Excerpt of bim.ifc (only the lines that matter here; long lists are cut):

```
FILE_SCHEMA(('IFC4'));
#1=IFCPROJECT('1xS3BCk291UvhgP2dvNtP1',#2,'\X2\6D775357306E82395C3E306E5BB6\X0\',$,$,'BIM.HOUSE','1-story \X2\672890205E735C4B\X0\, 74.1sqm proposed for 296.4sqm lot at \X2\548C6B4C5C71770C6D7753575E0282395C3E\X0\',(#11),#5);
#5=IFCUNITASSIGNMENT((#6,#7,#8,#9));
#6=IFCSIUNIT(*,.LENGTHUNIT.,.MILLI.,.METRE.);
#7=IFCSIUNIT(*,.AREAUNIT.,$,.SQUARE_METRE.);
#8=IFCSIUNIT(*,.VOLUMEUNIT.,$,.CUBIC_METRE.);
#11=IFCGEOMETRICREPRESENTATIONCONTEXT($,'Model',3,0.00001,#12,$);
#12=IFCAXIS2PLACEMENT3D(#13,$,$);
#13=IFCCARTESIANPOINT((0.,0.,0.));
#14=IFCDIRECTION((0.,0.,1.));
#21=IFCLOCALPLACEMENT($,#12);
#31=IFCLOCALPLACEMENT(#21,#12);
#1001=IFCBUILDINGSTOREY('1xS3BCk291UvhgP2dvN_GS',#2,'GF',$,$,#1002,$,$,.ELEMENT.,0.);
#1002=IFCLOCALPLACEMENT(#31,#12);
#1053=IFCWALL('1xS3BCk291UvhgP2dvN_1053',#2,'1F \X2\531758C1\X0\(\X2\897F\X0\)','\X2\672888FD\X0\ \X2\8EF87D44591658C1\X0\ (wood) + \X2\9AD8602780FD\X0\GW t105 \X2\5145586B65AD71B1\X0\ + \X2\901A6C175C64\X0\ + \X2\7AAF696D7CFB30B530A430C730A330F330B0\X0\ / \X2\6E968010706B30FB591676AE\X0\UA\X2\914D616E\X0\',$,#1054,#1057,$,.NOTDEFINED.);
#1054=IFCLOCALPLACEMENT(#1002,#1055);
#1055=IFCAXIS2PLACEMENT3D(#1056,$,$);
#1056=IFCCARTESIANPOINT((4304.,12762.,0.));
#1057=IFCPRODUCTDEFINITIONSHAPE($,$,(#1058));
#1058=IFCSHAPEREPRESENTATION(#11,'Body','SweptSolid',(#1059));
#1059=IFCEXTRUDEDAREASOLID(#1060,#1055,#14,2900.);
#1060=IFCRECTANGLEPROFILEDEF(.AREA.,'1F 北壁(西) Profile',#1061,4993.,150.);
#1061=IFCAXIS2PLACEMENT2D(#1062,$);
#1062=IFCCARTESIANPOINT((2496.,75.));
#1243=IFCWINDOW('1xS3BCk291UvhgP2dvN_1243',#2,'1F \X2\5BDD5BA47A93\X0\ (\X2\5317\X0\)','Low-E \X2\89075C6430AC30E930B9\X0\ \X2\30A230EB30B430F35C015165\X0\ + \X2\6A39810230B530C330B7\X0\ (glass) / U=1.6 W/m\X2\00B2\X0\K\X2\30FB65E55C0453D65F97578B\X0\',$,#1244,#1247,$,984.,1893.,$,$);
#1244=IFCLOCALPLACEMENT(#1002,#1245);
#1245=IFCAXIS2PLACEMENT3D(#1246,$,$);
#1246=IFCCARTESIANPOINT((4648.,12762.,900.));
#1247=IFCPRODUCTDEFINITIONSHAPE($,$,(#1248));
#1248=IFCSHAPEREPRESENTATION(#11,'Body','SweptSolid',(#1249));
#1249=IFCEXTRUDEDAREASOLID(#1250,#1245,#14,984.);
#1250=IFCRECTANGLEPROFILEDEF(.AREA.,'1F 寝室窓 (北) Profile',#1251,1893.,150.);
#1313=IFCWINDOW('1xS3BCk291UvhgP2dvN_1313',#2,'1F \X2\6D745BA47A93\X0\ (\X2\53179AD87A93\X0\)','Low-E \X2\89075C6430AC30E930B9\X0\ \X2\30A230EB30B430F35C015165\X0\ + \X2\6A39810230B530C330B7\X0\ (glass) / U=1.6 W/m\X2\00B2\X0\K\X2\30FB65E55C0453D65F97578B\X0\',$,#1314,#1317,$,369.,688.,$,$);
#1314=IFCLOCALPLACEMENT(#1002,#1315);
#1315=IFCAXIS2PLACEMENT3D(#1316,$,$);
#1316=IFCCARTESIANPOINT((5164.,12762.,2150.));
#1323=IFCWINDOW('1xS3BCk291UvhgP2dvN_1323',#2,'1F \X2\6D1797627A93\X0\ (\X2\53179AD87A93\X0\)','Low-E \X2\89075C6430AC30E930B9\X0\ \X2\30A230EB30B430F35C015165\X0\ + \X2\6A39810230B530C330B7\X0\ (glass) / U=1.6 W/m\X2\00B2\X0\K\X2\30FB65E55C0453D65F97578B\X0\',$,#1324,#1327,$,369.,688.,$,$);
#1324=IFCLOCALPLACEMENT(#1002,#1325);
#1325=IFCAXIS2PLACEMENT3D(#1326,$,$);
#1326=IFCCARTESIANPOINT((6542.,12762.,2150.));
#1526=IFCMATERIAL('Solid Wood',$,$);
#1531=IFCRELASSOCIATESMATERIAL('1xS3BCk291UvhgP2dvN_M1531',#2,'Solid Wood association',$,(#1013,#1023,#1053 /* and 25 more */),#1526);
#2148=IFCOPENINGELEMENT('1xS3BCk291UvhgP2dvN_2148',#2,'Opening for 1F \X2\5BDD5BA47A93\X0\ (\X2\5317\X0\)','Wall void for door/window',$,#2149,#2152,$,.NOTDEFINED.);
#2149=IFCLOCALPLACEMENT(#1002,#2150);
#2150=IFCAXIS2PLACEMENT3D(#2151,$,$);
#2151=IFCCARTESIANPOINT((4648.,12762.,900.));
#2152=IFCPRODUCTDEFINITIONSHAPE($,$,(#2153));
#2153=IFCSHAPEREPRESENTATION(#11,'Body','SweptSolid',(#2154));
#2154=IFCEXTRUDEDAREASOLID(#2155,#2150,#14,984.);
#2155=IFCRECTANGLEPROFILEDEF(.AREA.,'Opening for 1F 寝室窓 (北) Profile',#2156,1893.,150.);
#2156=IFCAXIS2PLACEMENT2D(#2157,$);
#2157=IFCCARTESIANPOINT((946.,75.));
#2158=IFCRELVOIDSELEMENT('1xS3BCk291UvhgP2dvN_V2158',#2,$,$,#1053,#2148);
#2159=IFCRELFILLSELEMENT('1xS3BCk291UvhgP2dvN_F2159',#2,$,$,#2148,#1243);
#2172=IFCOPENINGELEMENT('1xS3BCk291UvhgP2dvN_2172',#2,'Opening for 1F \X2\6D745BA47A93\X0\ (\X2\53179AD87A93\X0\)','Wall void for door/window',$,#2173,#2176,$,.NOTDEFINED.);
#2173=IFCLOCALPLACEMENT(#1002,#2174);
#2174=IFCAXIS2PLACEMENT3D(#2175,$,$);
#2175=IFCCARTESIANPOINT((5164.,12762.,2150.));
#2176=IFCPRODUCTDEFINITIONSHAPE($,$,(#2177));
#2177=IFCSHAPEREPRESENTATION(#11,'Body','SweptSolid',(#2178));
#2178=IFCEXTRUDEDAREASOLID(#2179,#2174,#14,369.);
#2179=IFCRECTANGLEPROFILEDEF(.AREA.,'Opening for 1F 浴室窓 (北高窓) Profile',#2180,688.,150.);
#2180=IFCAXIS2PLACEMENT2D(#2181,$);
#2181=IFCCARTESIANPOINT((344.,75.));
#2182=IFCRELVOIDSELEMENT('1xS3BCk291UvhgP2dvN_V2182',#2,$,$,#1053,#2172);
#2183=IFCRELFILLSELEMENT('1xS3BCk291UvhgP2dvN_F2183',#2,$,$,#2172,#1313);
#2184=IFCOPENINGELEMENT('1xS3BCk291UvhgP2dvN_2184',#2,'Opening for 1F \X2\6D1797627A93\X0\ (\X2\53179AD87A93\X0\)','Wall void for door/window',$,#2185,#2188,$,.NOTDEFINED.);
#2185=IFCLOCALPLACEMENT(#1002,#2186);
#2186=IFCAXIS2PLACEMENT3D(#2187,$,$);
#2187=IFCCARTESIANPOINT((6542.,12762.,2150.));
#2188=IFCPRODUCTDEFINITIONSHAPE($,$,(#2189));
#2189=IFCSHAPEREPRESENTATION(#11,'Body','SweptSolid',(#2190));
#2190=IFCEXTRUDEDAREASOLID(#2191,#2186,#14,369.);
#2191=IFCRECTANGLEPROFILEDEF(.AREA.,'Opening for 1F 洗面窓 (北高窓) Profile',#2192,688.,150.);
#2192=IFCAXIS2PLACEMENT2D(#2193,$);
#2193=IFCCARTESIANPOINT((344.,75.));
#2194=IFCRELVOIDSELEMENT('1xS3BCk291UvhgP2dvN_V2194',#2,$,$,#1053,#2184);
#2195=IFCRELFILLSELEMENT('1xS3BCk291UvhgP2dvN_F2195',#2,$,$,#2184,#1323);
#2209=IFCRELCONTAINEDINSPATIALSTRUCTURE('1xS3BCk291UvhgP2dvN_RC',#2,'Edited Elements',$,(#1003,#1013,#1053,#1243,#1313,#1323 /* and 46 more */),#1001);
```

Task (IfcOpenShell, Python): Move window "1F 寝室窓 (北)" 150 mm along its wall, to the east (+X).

```python
import ifcopenshell
import ifcopenshell.api.geometry
import ifcopenshell.util.placement
import ifcopenshell.util.unit

model = ifcopenshell.open("bim.ifc")
unit_scale = ifcopenshell.util.unit.calculate_unit_scale(model)

window = model.by_guid("1xS3BCk291UvhgP2dvN_1243")
opening = window.FillsVoids[0].RelatingOpeningElement
wall = opening.VoidsElements[0].RelatingBuildingElement

wall_matrix = ifcopenshell.util.placement.get_local_placement(wall.ObjectPlacement)
shift = wall_matrix[:3, 0] * 0.15 / unit_scale
before = ifcopenshell.util.placement.get_local_placement(window.ObjectPlacement)[:3, 3].copy()

# The window is not placed relative to its opening, so move both.
for product in (opening, window):
    matrix = ifcopenshell.util.placement.get_local_placement(product.ObjectPlacement)
    matrix[:3, 3] += shift
    ifcopenshell.api.geometry.edit_object_placement(model, product=product, matrix=matrix, is_si=False)

after = ifcopenshell.util.placement.get_local_placement(window.ObjectPlacement)[:3, 3]
print("window moved by", (after - before).round(3) + 0.0)

model.write("bim_edited.ifc")
```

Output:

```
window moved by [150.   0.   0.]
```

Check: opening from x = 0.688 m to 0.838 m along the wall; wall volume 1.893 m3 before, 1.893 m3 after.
